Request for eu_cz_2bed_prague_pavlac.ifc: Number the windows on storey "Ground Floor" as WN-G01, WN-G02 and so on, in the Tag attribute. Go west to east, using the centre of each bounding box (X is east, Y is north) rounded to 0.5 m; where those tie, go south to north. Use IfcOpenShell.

First a look at what the model holds.

```python
import ifcopenshell
import ifcopenshell.util.element
import ifcopenshell.util.placement

model = ifcopenshell.open("eu_cz_2bed_prague_pavlac.ifc")
print(model.schema)
storey = next(s for s in model.by_type("IfcBuildingStorey") if s.Name == "Ground Floor")
windows = [e for e in ifcopenshell.util.element.get_decomposition(storey) if e.is_a("IfcWindow")]
for e in sorted(windows, key=lambda e: e.id()):
    origin = ifcopenshell.util.placement.get_local_placement(e.ObjectPlacement)[:3, 3]
    print(e.id(), e.Tag, e.Name, origin.round(2) + 0.0, sep=" | ")
```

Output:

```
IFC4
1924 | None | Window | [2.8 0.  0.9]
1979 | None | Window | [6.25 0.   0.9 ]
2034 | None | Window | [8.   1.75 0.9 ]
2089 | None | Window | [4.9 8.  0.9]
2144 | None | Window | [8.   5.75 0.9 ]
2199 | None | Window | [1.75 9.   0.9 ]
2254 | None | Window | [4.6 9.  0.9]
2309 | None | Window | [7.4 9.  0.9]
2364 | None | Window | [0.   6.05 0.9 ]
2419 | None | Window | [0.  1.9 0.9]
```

```python
import ifcopenshell
import ifcopenshell.geom
import ifcopenshell.util.element
import ifcopenshell.util.shape

model = ifcopenshell.open("eu_cz_2bed_prague_pavlac.ifc")
settings = ifcopenshell.geom.settings()
settings.set("use-world-coords", True)


def centre(element):
    shape = ifcopenshell.geom.create_shape(settings, element)
    return ifcopenshell.util.shape.get_bbox_centroid(shape.geometry)


storey = next(s for s in model.by_type("IfcBuildingStorey") if s.Name == "Ground Floor")
windows = [e for e in ifcopenshell.util.element.get_decomposition(storey) if e.is_a("IfcWindow")]

# Insertion points can sit at a corner or the storey origin, so sort by the geometry (in metres).
centres = {e: centre(e) for e in windows}
windows.sort(key=lambda e: (round(centres[e][0] / 0.5), centres[e][1]))

for i, e in enumerate(windows, start=1):
    number = f"WN-G{i:02d}"
    e.Tag = number
    print(e.id(), number)

model.write("eu_cz_2bed_prague_pavlac_edited.ifc")
```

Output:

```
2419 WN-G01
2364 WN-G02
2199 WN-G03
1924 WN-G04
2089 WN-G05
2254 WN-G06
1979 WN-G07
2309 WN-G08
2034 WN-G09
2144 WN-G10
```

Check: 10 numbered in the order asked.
